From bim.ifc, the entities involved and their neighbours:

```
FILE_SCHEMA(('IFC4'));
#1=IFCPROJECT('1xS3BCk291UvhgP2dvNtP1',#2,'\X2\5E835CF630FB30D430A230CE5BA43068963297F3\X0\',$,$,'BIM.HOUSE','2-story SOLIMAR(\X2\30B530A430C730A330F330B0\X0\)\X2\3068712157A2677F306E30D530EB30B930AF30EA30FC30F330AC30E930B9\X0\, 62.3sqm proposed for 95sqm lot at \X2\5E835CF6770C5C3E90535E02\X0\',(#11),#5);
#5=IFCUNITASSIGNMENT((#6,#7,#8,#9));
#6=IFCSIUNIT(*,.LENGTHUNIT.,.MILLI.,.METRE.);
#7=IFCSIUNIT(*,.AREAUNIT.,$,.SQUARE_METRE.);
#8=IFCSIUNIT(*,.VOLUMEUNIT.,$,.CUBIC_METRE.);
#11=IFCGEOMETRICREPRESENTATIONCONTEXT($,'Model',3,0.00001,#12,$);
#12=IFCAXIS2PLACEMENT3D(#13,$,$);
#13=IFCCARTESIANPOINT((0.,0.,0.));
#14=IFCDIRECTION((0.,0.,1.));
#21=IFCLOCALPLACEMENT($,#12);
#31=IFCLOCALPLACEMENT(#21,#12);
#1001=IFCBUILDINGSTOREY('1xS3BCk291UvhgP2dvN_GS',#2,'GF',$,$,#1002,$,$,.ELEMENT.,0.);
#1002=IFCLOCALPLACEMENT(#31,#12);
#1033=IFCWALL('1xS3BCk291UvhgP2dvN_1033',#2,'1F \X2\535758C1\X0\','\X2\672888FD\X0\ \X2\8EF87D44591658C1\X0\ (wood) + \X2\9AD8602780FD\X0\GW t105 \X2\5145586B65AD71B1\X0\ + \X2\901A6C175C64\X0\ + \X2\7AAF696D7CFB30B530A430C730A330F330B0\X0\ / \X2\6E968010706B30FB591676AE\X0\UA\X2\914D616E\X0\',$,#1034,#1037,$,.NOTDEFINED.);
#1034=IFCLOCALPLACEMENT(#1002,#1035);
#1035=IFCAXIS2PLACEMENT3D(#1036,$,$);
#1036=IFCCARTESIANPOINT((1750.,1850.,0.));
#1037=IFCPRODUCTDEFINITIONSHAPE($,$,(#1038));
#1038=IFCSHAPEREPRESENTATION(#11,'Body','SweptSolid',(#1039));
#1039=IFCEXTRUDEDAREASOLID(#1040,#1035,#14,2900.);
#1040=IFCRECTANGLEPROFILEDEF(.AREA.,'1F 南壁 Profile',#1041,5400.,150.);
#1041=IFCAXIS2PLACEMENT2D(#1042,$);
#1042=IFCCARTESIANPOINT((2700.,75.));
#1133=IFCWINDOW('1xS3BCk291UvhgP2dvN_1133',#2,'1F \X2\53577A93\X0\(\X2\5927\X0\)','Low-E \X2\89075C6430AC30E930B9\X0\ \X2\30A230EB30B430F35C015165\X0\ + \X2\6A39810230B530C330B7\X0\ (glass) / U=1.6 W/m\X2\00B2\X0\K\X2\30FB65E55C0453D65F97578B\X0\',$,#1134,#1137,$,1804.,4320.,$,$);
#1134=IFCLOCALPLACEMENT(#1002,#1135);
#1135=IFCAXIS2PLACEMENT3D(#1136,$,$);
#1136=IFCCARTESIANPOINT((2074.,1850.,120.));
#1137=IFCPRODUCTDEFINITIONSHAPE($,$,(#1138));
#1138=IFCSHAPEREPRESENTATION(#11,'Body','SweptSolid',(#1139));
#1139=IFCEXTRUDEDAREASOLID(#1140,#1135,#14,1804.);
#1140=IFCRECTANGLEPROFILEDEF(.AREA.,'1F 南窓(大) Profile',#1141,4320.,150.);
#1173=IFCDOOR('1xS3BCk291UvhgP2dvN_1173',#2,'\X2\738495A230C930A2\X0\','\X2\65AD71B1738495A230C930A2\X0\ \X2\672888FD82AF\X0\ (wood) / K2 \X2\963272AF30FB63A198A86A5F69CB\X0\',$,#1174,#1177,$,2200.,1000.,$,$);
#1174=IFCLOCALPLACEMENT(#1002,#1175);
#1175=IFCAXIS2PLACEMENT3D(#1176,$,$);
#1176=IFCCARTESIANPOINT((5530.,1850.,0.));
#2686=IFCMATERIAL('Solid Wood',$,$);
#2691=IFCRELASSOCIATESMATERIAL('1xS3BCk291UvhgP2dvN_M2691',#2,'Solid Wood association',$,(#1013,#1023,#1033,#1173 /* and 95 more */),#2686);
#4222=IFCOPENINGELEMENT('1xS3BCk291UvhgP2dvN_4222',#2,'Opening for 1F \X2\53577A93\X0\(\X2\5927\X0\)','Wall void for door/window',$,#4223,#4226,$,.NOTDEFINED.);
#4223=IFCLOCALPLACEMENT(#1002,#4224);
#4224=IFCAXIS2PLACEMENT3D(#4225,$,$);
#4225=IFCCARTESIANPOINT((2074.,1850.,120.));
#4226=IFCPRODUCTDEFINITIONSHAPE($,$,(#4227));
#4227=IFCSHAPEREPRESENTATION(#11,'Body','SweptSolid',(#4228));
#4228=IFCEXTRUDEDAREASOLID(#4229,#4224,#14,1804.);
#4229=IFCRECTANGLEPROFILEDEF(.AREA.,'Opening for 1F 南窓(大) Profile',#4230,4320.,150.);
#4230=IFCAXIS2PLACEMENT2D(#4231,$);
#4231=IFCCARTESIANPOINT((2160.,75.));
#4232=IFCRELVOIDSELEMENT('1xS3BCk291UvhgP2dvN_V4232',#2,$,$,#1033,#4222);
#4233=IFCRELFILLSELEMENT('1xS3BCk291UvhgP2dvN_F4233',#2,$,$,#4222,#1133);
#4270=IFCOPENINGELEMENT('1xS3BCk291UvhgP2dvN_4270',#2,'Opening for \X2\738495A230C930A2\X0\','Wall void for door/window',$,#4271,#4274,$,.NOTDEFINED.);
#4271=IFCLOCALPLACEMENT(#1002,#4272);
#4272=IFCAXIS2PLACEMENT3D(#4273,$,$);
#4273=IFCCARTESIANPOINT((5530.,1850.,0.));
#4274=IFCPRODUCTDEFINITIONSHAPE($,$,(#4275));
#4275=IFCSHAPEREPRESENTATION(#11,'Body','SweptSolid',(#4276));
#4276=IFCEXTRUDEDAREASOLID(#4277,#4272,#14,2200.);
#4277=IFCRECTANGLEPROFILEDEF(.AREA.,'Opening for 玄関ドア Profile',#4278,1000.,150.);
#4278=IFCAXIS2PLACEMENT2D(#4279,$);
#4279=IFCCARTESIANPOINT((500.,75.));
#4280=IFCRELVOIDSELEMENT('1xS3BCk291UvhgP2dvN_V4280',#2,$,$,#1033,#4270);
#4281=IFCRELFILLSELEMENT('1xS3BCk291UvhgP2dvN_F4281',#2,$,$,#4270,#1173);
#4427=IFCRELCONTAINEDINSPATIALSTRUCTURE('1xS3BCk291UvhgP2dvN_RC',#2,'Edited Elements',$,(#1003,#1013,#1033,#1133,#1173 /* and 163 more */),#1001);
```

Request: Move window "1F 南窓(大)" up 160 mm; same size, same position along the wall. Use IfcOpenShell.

```python
import numpy as np
import ifcopenshell
import ifcopenshell.api.geometry
import ifcopenshell.util.placement
import ifcopenshell.util.unit

model = ifcopenshell.open("bim.ifc")
unit_scale = ifcopenshell.util.unit.calculate_unit_scale(model)

window = model.by_guid("1xS3BCk291UvhgP2dvN_1133")
opening = window.FillsVoids[0].RelatingOpeningElement
dz = 0.16 / unit_scale

shift = np.array([0.0, 0.0, dz])
# The window is not placed relative to its opening, so move both.
for product in (opening, window):
    matrix = ifcopenshell.util.placement.get_local_placement(product.ObjectPlacement)
    matrix[:3, 3] += shift
    ifcopenshell.api.geometry.edit_object_placement(model, product=product, matrix=matrix, is_si=False)

print(f"moved by {dz * unit_scale:+.3f} m")

model.write("bim_v2.ifc")
```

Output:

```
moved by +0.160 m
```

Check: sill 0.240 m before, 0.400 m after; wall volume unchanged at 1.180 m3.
